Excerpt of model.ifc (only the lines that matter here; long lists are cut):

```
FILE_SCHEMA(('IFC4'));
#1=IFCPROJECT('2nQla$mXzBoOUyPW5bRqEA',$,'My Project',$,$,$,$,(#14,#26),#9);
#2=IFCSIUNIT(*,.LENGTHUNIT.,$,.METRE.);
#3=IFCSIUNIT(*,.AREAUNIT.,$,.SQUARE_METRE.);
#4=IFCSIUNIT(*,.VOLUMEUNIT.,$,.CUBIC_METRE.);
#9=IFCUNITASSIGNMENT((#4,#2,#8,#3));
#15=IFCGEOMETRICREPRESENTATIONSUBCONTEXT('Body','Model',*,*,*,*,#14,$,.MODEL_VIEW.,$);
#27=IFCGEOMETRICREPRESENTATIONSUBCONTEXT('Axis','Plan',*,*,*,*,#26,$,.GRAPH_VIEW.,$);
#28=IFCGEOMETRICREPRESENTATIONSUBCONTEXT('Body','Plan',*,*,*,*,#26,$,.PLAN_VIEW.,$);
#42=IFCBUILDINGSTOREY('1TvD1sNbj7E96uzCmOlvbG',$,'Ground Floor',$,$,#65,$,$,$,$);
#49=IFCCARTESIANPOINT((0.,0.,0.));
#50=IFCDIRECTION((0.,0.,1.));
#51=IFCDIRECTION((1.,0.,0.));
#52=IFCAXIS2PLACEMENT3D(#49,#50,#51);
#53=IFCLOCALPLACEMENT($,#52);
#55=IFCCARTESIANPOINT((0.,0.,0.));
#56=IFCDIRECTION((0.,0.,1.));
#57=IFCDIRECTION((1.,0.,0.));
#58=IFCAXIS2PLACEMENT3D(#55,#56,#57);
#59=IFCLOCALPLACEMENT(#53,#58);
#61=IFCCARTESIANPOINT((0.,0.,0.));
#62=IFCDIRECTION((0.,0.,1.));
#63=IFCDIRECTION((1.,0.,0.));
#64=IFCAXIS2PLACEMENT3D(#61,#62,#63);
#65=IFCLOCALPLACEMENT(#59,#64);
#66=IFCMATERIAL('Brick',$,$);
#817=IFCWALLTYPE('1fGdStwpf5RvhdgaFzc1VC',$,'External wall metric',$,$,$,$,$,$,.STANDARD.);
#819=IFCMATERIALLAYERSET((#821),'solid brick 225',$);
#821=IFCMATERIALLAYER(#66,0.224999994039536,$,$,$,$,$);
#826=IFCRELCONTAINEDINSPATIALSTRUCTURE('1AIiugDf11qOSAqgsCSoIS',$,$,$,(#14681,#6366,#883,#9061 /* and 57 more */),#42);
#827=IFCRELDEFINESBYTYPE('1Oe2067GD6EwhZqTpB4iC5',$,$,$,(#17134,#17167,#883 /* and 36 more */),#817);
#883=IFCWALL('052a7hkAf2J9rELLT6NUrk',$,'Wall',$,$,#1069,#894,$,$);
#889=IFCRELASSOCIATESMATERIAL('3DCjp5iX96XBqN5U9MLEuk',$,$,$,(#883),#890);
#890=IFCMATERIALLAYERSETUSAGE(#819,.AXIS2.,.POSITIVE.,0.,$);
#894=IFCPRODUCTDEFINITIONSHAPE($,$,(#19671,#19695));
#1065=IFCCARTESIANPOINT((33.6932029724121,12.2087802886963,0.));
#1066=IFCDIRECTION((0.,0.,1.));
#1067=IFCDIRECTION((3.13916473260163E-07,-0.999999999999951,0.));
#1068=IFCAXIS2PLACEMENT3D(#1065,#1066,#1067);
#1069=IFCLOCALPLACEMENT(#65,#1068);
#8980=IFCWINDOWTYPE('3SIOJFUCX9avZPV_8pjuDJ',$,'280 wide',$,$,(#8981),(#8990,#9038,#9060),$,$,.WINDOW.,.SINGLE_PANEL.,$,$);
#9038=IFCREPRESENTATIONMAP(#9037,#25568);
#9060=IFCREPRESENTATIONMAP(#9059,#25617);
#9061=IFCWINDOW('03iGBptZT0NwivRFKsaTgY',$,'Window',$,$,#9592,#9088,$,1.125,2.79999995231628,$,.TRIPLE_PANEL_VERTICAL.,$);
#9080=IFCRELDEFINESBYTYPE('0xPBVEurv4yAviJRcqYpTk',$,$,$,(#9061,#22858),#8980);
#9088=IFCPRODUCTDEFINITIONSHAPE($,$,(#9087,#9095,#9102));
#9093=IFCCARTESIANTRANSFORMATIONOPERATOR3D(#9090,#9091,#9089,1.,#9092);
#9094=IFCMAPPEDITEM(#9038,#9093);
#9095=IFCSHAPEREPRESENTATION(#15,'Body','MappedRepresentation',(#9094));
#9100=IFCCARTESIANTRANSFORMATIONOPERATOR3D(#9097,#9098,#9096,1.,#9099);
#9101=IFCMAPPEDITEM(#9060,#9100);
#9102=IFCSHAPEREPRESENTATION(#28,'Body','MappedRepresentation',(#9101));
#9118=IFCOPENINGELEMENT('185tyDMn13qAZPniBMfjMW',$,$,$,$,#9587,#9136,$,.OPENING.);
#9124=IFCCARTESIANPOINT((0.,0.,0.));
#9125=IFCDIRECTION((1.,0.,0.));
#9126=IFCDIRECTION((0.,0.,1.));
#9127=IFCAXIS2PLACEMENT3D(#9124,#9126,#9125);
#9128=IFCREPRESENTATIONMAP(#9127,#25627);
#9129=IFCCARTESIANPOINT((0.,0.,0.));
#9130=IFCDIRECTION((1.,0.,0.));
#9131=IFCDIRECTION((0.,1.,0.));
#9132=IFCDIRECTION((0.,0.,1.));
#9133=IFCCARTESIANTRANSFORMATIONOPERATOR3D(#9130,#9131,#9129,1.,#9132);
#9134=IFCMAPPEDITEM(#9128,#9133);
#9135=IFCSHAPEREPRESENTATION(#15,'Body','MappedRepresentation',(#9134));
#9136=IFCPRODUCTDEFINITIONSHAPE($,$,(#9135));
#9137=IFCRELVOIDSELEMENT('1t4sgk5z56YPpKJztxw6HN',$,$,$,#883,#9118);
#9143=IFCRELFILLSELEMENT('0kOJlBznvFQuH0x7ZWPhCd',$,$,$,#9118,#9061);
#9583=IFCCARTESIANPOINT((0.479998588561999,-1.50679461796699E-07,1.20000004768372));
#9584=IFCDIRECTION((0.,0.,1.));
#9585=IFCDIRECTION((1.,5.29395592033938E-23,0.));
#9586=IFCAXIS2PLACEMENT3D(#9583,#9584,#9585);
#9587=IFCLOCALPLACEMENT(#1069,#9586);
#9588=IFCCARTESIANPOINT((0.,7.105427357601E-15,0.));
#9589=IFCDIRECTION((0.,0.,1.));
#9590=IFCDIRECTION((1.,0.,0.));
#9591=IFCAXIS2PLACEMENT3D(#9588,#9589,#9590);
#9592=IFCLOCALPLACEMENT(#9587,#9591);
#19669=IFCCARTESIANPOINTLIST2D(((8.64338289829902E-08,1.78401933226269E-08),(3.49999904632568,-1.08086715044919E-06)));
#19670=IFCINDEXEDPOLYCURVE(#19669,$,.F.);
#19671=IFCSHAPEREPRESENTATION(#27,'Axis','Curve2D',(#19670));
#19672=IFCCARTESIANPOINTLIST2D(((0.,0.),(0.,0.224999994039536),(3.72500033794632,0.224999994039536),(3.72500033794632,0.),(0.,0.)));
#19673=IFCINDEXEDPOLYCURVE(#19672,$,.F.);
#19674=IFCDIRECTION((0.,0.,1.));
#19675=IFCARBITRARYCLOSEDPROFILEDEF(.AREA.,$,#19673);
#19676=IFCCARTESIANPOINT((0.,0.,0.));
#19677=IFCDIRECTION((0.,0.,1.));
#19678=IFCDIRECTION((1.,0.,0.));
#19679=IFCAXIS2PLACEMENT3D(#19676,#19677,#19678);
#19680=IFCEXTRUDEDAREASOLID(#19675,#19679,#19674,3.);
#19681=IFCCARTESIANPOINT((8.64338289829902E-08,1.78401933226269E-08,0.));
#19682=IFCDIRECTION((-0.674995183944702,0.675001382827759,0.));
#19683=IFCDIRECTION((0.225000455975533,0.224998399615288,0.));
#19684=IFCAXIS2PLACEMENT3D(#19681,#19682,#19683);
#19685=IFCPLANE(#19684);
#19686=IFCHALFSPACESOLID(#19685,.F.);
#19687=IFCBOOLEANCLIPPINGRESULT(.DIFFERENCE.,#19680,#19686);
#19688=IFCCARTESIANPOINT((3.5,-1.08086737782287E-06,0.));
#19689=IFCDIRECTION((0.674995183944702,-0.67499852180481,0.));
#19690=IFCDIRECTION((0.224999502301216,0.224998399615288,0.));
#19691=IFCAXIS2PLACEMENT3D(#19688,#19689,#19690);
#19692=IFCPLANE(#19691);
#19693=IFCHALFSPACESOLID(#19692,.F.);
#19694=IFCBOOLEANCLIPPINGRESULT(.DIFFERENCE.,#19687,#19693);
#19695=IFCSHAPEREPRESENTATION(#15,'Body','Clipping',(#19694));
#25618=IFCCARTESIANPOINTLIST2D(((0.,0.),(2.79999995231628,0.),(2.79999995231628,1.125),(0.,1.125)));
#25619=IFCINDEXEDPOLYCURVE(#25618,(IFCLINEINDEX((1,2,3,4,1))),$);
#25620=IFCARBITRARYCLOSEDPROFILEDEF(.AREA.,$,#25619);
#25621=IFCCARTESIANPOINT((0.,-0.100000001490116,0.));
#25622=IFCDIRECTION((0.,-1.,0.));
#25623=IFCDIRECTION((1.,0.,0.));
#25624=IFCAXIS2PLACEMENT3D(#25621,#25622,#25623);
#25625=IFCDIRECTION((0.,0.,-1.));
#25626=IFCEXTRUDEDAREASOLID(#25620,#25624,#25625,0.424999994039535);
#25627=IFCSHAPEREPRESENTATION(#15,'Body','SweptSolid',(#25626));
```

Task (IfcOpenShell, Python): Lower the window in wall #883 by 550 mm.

```python
import numpy as np
import ifcopenshell
import ifcopenshell.api.geometry
import ifcopenshell.util.placement
import ifcopenshell.util.unit

model = ifcopenshell.open("model.ifc")
unit_scale = ifcopenshell.util.unit.calculate_unit_scale(model)

window = model.by_id(9061)
opening = window.FillsVoids[0].RelatingOpeningElement
dz = -0.55

shift = np.array([0.0, 0.0, dz])
# The window is placed relative to its opening, so it follows when the opening moves.
matrix = ifcopenshell.util.placement.get_local_placement(opening.ObjectPlacement)
matrix[:3, 3] += shift
ifcopenshell.api.geometry.edit_object_placement(
    model, product=opening, matrix=matrix, is_si=False, should_transform_children=True
)

print(f"moved by {dz * unit_scale:+.3f} m")

model.write("model_v2.ifc")
```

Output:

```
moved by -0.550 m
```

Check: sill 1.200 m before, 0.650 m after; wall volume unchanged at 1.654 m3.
